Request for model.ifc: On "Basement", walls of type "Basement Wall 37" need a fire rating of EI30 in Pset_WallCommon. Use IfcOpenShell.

First a look at what the model holds.

```python
import ifcopenshell
import ifcopenshell.util.element

model = ifcopenshell.open("model.ifc")
print(model.schema)
storey = next(s for s in model.by_type("IfcBuildingStorey") if s.Name == "Basement")
walls = [e for e in ifcopenshell.util.element.get_decomposition(storey) if e.is_a("IfcWall")]
seen = {}
for e in walls:
    element_type = ifcopenshell.util.element.get_type(e)
    key = (element_type.Name if element_type != e and element_type else None, ifcopenshell.util.element.get_pset(e, "Pset_WallCommon", "FireRating"))
    seen[key] = seen.get(key, 0) + 1
for (name, value), count in sorted(seen.items(), key=str):
    print(count, "x", name, "|", value)
```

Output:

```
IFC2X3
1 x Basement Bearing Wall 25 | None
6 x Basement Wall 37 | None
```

```python
import ifcopenshell
import ifcopenshell.api.pset
import ifcopenshell.util.element

model = ifcopenshell.open("model.ifc")

storey = next(s for s in model.by_type("IfcBuildingStorey") if s.Name == "Basement")
walls = [e for e in ifcopenshell.util.element.get_decomposition(storey) if e.is_a("IfcWall")]

count = 0
for e in walls:
    element_type = ifcopenshell.util.element.get_type(e)
    if element_type in (None, e) or element_type.Name != "Basement Wall 37":
        continue
    # add_pset returns the element's existing set when there is one.
    pset = ifcopenshell.api.pset.add_pset(model, product=e, name="Pset_WallCommon")
    ifcopenshell.api.pset.edit_pset(model, pset=pset, properties={"FireRating": "EI30"})
    count += 1

print(count, "walls updated")

model.write("model_v2.ifc")
```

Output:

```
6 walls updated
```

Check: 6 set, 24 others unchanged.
